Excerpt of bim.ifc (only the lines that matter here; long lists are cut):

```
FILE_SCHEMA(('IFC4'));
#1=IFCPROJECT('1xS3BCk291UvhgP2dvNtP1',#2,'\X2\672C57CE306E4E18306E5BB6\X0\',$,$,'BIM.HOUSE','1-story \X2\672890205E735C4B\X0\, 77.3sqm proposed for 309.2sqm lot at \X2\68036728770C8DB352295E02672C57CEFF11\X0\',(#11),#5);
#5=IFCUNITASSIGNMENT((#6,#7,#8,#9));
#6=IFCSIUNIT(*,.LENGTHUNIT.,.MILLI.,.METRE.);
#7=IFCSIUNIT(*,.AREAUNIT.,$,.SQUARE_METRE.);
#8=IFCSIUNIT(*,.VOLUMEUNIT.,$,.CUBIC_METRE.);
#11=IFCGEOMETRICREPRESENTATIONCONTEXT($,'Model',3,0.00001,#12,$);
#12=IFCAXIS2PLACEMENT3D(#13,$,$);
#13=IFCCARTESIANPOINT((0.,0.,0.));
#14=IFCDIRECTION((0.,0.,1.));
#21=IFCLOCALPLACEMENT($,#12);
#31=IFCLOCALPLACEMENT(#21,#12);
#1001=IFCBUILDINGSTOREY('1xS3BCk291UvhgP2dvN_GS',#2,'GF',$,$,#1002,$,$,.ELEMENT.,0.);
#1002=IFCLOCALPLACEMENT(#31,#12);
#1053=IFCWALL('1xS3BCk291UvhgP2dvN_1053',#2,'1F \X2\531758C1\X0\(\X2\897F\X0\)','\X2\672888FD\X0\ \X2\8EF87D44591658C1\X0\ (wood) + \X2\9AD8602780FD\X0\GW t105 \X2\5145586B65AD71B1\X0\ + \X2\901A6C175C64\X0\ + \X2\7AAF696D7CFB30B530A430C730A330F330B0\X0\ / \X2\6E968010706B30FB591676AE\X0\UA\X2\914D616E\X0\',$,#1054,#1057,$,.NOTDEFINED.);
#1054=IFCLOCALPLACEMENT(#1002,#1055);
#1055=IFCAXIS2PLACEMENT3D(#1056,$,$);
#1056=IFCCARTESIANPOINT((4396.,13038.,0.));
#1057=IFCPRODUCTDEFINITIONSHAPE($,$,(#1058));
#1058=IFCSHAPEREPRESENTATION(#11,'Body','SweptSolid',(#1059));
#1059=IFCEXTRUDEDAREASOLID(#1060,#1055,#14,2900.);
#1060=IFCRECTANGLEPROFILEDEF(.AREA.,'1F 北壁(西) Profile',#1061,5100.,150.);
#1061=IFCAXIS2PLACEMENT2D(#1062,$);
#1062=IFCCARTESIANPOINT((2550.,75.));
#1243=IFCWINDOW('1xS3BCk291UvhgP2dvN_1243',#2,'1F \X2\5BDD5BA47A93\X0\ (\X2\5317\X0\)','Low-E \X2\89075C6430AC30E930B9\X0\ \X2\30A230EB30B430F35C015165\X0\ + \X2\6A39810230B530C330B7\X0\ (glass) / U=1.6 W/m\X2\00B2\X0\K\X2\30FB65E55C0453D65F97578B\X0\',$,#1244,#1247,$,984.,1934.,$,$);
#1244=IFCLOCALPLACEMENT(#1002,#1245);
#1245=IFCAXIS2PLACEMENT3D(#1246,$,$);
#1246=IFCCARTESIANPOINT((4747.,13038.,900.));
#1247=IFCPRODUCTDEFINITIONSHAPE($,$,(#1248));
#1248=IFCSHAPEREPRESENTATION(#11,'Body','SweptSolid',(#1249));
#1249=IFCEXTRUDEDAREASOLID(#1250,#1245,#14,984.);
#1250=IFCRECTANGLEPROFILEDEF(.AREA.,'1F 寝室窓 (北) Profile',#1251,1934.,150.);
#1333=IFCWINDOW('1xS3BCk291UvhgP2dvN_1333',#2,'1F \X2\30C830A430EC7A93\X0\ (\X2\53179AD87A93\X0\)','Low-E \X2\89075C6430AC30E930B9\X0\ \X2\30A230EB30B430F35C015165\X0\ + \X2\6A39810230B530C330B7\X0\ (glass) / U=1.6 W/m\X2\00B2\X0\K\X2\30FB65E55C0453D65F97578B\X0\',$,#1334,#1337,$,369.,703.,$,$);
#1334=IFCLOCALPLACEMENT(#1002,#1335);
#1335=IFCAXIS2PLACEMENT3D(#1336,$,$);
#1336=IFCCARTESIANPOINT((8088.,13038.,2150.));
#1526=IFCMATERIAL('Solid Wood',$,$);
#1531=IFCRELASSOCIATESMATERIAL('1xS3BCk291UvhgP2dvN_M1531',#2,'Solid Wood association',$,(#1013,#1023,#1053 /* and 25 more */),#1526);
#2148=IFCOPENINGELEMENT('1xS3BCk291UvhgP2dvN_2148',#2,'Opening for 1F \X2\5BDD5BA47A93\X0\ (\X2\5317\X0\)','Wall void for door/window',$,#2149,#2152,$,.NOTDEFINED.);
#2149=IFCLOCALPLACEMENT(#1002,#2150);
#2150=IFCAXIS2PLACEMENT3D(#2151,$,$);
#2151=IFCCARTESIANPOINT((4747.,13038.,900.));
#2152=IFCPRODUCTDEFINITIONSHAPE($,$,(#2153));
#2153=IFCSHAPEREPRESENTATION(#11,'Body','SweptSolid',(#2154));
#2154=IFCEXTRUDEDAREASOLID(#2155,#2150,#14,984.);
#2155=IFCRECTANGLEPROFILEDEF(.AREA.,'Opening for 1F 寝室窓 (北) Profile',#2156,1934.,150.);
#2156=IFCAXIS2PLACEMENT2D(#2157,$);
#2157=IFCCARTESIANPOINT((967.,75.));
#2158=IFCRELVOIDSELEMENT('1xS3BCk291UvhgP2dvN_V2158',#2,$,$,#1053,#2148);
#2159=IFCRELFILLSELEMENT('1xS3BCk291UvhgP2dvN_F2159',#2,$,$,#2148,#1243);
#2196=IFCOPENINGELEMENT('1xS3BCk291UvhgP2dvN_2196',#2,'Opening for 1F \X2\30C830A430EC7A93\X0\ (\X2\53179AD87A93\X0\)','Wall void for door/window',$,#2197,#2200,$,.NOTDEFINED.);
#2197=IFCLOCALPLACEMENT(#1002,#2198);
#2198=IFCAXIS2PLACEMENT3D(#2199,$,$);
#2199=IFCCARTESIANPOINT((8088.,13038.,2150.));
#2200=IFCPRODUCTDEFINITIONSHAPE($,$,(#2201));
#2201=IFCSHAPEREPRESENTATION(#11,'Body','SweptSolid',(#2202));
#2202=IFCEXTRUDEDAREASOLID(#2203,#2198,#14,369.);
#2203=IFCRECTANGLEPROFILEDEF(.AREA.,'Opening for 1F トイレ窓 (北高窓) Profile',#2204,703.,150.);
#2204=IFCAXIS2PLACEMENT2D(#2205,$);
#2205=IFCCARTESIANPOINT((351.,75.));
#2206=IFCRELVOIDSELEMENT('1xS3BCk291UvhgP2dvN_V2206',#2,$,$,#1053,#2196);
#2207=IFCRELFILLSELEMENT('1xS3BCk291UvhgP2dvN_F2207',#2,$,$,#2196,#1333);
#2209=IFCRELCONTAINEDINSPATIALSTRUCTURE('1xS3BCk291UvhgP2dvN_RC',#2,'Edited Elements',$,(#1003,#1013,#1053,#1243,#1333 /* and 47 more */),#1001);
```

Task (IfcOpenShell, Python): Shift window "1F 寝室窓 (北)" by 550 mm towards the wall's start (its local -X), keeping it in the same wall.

```python
import ifcopenshell
import ifcopenshell.api.geometry
import ifcopenshell.util.placement
import ifcopenshell.util.unit

model = ifcopenshell.open("bim.ifc")
unit_scale = ifcopenshell.util.unit.calculate_unit_scale(model)

window = model.by_guid("1xS3BCk291UvhgP2dvN_1243")
opening = window.FillsVoids[0].RelatingOpeningElement
wall = opening.VoidsElements[0].RelatingBuildingElement

wall_matrix = ifcopenshell.util.placement.get_local_placement(wall.ObjectPlacement)
shift = wall_matrix[:3, 0] * -0.55 / unit_scale
before = ifcopenshell.util.placement.get_local_placement(window.ObjectPlacement)[:3, 3].copy()

# The window is not placed relative to its opening, so move both.
for product in (opening, window):
    matrix = ifcopenshell.util.placement.get_local_placement(product.ObjectPlacement)
    matrix[:3, 3] += shift
    ifcopenshell.api.geometry.edit_object_placement(model, product=product, matrix=matrix, is_si=False)

after = ifcopenshell.util.placement.get_local_placement(window.ObjectPlacement)[:3, 3]
print("window moved by", (after - before).round(3) + 0.0)

model.write("bim_edited.ifc")
```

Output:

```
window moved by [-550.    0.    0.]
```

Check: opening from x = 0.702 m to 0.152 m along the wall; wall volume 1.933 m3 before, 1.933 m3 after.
